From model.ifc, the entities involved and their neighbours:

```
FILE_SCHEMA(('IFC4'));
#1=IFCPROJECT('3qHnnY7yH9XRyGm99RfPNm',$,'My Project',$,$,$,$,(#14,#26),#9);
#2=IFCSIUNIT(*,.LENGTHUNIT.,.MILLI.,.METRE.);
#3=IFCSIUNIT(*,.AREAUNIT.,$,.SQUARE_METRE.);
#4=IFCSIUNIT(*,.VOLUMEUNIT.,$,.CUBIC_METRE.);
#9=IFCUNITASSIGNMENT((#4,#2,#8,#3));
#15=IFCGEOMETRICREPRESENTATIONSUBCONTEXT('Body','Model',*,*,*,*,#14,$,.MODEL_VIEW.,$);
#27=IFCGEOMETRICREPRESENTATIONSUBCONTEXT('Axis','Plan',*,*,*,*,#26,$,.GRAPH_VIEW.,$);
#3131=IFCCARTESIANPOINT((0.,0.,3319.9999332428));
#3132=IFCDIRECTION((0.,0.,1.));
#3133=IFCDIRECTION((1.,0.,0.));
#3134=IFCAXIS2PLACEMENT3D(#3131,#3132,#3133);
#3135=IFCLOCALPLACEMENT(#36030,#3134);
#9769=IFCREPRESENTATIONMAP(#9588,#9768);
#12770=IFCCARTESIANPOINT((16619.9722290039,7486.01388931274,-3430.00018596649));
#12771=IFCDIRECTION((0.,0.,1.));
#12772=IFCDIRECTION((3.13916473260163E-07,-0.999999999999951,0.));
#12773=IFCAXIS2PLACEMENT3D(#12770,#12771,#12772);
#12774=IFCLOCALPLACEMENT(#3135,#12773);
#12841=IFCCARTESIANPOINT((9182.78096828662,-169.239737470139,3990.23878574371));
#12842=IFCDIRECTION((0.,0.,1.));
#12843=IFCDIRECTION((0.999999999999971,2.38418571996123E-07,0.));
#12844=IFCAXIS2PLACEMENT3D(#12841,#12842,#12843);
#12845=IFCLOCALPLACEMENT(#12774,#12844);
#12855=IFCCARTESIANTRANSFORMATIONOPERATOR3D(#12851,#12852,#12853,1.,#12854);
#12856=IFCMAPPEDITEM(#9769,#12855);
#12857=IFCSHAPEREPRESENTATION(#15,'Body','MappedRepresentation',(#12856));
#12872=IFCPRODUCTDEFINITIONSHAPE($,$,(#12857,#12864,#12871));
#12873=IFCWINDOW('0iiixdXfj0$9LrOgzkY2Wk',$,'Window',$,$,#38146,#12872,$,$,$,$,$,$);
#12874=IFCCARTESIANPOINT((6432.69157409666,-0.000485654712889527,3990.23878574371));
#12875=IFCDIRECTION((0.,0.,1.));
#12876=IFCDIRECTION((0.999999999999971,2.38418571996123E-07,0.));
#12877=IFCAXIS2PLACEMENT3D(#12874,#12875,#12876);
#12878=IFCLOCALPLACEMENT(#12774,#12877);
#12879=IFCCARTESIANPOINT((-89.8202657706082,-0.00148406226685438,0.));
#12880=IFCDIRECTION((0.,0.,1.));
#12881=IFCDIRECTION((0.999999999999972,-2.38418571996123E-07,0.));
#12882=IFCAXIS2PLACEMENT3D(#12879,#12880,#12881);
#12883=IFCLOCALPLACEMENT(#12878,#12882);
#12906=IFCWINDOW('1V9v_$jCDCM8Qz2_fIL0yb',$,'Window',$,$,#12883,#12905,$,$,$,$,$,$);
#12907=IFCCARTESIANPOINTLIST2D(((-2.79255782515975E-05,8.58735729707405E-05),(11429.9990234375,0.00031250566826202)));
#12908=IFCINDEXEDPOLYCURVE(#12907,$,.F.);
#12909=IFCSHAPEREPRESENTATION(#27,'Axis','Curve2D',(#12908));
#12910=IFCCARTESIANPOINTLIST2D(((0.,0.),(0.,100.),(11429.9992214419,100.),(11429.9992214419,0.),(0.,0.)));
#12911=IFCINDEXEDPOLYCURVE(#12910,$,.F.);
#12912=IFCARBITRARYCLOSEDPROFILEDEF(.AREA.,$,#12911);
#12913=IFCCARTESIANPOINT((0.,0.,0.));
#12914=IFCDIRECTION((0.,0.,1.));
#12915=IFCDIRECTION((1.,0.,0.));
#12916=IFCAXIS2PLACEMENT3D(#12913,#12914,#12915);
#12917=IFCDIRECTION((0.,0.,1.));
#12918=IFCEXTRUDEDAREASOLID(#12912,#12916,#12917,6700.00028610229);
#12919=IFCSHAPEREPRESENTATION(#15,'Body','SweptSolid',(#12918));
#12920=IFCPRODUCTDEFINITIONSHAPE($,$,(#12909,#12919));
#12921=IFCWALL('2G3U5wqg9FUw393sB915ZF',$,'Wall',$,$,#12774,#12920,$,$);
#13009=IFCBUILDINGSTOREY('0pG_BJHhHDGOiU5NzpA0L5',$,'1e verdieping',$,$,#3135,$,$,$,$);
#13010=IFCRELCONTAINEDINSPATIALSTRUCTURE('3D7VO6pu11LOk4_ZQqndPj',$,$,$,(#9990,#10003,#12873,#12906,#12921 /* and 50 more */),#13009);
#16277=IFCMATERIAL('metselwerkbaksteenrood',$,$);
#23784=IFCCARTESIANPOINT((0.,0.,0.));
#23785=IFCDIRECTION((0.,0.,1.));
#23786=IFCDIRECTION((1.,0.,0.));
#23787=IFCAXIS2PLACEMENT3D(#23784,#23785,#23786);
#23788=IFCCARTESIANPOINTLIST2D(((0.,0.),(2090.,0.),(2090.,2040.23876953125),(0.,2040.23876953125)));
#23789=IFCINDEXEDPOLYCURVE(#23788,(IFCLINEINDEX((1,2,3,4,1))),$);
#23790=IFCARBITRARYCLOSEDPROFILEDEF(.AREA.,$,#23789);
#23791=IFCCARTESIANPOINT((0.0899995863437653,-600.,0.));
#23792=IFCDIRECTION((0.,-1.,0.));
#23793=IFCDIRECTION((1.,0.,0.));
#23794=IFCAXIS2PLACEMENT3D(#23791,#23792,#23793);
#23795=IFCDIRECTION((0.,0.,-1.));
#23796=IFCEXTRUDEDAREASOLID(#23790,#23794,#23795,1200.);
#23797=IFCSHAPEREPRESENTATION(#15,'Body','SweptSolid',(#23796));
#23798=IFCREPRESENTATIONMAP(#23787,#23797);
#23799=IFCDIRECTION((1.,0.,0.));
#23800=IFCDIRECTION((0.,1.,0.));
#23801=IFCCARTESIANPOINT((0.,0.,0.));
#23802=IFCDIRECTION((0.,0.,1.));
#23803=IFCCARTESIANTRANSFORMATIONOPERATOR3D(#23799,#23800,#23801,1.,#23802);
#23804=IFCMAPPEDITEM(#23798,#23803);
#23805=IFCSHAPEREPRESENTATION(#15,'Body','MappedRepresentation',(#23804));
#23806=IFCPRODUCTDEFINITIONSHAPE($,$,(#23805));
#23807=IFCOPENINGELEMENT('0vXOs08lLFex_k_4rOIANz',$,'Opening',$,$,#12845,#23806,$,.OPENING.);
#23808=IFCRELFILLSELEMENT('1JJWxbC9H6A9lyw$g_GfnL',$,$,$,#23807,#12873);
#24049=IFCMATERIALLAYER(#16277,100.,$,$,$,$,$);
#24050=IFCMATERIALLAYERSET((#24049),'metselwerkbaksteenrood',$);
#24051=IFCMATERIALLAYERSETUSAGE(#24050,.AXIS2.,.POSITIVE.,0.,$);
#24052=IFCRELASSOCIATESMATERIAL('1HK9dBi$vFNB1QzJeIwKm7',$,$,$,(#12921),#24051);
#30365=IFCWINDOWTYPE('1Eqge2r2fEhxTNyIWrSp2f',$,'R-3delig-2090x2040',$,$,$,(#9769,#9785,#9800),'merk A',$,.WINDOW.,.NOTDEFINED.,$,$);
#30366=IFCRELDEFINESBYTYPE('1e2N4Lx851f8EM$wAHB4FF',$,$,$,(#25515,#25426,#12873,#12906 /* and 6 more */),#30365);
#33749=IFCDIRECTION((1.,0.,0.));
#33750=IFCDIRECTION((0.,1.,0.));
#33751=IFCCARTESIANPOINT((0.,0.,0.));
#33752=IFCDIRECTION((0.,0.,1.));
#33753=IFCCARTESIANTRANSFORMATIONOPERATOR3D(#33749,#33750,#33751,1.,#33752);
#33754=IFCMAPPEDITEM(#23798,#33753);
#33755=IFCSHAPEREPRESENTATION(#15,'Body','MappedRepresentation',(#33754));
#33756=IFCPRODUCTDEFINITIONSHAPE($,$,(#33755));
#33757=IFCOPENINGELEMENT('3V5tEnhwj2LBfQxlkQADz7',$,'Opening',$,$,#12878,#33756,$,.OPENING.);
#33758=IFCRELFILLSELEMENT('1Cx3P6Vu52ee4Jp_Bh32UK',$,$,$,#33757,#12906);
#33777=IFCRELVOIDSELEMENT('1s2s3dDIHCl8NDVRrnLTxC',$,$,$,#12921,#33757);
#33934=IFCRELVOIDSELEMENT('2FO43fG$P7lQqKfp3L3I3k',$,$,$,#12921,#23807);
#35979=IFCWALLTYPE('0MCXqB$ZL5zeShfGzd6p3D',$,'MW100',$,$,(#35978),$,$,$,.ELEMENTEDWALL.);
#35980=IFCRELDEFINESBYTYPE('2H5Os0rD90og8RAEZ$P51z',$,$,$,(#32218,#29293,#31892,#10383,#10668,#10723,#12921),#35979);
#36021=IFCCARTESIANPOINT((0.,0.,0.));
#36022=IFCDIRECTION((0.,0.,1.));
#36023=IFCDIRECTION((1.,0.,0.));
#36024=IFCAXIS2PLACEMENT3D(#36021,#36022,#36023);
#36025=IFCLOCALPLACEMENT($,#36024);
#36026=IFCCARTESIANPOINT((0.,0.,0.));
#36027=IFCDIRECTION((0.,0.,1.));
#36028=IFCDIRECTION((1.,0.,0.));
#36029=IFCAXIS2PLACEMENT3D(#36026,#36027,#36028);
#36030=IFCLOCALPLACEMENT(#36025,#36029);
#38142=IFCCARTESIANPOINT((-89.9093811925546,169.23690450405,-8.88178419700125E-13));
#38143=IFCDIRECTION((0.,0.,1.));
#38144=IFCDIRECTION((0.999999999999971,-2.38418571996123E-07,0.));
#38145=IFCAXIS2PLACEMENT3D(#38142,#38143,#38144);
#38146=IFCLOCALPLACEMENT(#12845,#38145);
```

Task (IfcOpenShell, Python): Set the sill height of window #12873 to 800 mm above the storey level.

```python
import numpy as np
import ifcopenshell
import ifcopenshell.api.geometry
import ifcopenshell.geom
import ifcopenshell.util.element
import ifcopenshell.util.placement
import ifcopenshell.util.shape
import ifcopenshell.util.unit

model = ifcopenshell.open("model.ifc")
unit_scale = ifcopenshell.util.unit.calculate_unit_scale(model)

window = model.by_guid("0iiixdXfj0$9LrOgzkY2Wk")
opening = window.FillsVoids[0].RelatingOpeningElement
storey = ifcopenshell.util.element.get_container(window, ifc_class="IfcBuildingStorey")
level = ifcopenshell.util.placement.get_local_placement(storey.ObjectPlacement)[2, 3]

# The opening's origin need not be at the sill, so measure its lowest point.
shape = ifcopenshell.geom.create_shape(ifcopenshell.geom.settings(), opening)
bottom = ifcopenshell.util.shape.get_shape_bottom_elevation(shape, shape.geometry) / unit_scale
dz = level + 0.8 / unit_scale - bottom

shift = np.array([0.0, 0.0, dz])
# The window is placed relative to its opening, so it follows when the opening moves.
matrix = ifcopenshell.util.placement.get_local_placement(opening.ObjectPlacement)
matrix[:3, 3] += shift
ifcopenshell.api.geometry.edit_object_placement(
    model, product=opening, matrix=matrix, is_si=False, should_transform_children=True
)

print(f"moved by {dz * unit_scale:+.3f} m")

model.write("model_updated.ifc")
```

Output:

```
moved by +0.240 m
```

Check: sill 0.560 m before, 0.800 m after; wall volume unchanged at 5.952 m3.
